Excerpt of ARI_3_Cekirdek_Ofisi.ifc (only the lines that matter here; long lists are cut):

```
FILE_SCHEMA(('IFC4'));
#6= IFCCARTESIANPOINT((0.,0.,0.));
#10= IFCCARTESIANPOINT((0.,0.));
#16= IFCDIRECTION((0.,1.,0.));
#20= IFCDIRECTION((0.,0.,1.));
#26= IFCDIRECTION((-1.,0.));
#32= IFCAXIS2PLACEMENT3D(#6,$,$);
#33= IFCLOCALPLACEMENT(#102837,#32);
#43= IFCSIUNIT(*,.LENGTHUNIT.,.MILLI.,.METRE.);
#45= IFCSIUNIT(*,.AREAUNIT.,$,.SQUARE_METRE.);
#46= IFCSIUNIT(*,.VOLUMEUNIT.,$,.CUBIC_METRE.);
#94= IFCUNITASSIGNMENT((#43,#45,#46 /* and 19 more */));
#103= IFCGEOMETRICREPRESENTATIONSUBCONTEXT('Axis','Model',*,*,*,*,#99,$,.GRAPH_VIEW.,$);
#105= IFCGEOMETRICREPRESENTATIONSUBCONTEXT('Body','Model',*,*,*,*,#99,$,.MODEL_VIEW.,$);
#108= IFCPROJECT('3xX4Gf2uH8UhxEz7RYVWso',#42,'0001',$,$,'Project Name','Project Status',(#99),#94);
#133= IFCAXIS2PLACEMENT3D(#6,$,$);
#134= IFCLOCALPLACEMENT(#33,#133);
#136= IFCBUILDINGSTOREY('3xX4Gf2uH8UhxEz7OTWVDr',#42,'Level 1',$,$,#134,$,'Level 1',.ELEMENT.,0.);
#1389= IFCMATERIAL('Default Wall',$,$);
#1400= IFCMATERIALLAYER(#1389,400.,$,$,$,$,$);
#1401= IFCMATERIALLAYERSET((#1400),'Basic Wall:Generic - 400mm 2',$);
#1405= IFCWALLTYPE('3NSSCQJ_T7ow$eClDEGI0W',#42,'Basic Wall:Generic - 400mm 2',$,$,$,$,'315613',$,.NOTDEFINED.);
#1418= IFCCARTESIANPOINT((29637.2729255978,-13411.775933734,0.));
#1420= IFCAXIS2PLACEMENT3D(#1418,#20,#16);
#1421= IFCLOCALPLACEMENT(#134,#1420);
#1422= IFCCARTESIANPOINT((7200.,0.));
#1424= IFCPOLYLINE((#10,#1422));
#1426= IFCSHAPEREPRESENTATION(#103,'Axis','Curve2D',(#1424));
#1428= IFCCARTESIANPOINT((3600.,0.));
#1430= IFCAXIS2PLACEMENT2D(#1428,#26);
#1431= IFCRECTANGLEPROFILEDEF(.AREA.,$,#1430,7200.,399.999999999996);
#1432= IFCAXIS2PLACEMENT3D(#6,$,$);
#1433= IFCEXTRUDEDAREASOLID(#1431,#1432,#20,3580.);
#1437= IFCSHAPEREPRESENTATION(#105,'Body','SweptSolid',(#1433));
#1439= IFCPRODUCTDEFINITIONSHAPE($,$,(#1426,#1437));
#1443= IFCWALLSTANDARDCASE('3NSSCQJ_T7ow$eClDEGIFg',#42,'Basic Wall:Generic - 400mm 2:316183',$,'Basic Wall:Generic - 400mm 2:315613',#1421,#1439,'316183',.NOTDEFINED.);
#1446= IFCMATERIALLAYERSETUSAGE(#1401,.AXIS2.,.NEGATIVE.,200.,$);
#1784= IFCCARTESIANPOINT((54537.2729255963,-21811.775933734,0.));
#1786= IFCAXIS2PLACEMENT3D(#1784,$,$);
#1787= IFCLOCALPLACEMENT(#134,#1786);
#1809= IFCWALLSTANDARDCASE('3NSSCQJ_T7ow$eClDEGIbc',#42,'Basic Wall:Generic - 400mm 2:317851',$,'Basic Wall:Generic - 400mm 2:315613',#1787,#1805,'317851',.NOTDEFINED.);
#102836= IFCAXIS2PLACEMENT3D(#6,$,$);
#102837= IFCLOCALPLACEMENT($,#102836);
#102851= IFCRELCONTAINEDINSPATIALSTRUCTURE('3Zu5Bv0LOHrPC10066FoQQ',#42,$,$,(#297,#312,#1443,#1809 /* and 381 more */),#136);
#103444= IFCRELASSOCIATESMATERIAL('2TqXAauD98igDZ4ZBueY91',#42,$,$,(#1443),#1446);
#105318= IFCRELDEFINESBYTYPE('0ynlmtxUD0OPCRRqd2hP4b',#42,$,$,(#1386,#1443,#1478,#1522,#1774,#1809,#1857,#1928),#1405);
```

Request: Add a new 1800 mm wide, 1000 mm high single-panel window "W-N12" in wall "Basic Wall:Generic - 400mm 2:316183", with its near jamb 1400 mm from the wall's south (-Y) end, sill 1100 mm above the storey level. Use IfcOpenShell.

```python
import numpy as np
import ifcopenshell
import ifcopenshell.api.feature
import ifcopenshell.api.geometry
import ifcopenshell.api.root
import ifcopenshell.api.spatial
import ifcopenshell.geom
import ifcopenshell.util.element
import ifcopenshell.util.placement
import ifcopenshell.util.representation
import ifcopenshell.util.shape
import ifcopenshell.util.unit

model = ifcopenshell.open("ARI_3_Cekirdek_Ofisi.ifc")
unit_scale = ifcopenshell.util.unit.calculate_unit_scale(model)
settings = ifcopenshell.geom.settings()


def volume(element):
    """Net volume in cubic metres, openings subtracted."""
    shape = ifcopenshell.geom.create_shape(settings, element)
    return ifcopenshell.util.shape.get_volume(shape.geometry)


wall = model.by_guid("3NSSCQJ_T7ow$eClDEGIFg")
storey = ifcopenshell.util.element.get_container(wall, ifc_class="IfcBuildingStorey")
context = ifcopenshell.util.representation.get_context(model, "Model", "Body", "MODEL_VIEW")
before = volume(wall)

width, height, from_end, sill = 1.8, 1, 1.4, 1.1  # metres

# The wall runs along its own X axis, and the end named is its -X end.
wall_shape = ifcopenshell.geom.create_shape(settings, wall)
x, y, z = ifcopenshell.util.shape.get_vertices(wall_shape.geometry).T
start = x.min() + from_end
face, thickness = float(y.min()), float(y.max() - y.min())
wall_matrix = ifcopenshell.util.placement.get_local_placement(wall.ObjectPlacement)
level = ifcopenshell.util.placement.get_local_placement(storey.ObjectPlacement)[2, 3]


def in_wall(x, y):
    """Placement at x, y metres in the wall's axes, at sill height."""
    matrix = wall_matrix.copy()
    matrix[:, 3] = wall_matrix @ np.array([x / unit_scale, y / unit_scale, 0.0, 1.0])
    matrix[2, 3] = level + sill / unit_scale
    return matrix


# Opening: a box that overshoots both wall faces by 50 mm.
opening = ifcopenshell.api.root.create_entity(model, ifc_class="IfcOpeningElement", predefined_type="OPENING")
box = ifcopenshell.api.geometry.add_wall_representation(
    model, context=context, length=width, height=height, thickness=thickness + 0.1
)
ifcopenshell.api.geometry.assign_representation(model, product=opening, representation=box)
ifcopenshell.api.geometry.edit_object_placement(model, product=opening, matrix=in_wall(start, face - 0.05), is_si=False)
ifcopenshell.api.feature.add_feature(model, feature=opening, element=wall)

window = ifcopenshell.api.root.create_entity(model, ifc_class="IfcWindow", name="W-N12", predefined_type="WINDOW")
window.OverallWidth, window.OverallHeight = width / unit_scale, height / unit_scale
window.PartitioningType = "SINGLE_PANEL"
body = ifcopenshell.api.geometry.add_window_representation(
    model,
    context=context,
    overall_width=window.OverallWidth,
    overall_height=window.OverallHeight,
    partition_type="SINGLE_PANEL",
)
ifcopenshell.api.geometry.assign_representation(model, product=window, representation=body)
ifcopenshell.api.spatial.assign_container(model, products=[window], relating_structure=storey)
ifcopenshell.api.feature.add_filling(model, opening=opening, element=window)

# Centre the window in the wall's thickness.
ifcopenshell.api.geometry.edit_object_placement(model, product=window, matrix=in_wall(start, face), is_si=False)
window_shape = ifcopenshell.geom.create_shape(settings, window)
depth = ifcopenshell.util.shape.get_vertices(window_shape.geometry)[:, 1]
offset = face + thickness / 2 - (depth.min() + depth.max()) / 2
ifcopenshell.api.geometry.edit_object_placement(model, product=window, matrix=in_wall(start, offset), is_si=False)

after = volume(wall)

print(f"wall volume {before:.3f} -> {after:.3f} m3")

model.write("ARI_3_Cekirdek_Ofisi-out.ifc")
```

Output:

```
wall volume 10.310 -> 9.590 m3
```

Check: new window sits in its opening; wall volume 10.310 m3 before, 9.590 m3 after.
